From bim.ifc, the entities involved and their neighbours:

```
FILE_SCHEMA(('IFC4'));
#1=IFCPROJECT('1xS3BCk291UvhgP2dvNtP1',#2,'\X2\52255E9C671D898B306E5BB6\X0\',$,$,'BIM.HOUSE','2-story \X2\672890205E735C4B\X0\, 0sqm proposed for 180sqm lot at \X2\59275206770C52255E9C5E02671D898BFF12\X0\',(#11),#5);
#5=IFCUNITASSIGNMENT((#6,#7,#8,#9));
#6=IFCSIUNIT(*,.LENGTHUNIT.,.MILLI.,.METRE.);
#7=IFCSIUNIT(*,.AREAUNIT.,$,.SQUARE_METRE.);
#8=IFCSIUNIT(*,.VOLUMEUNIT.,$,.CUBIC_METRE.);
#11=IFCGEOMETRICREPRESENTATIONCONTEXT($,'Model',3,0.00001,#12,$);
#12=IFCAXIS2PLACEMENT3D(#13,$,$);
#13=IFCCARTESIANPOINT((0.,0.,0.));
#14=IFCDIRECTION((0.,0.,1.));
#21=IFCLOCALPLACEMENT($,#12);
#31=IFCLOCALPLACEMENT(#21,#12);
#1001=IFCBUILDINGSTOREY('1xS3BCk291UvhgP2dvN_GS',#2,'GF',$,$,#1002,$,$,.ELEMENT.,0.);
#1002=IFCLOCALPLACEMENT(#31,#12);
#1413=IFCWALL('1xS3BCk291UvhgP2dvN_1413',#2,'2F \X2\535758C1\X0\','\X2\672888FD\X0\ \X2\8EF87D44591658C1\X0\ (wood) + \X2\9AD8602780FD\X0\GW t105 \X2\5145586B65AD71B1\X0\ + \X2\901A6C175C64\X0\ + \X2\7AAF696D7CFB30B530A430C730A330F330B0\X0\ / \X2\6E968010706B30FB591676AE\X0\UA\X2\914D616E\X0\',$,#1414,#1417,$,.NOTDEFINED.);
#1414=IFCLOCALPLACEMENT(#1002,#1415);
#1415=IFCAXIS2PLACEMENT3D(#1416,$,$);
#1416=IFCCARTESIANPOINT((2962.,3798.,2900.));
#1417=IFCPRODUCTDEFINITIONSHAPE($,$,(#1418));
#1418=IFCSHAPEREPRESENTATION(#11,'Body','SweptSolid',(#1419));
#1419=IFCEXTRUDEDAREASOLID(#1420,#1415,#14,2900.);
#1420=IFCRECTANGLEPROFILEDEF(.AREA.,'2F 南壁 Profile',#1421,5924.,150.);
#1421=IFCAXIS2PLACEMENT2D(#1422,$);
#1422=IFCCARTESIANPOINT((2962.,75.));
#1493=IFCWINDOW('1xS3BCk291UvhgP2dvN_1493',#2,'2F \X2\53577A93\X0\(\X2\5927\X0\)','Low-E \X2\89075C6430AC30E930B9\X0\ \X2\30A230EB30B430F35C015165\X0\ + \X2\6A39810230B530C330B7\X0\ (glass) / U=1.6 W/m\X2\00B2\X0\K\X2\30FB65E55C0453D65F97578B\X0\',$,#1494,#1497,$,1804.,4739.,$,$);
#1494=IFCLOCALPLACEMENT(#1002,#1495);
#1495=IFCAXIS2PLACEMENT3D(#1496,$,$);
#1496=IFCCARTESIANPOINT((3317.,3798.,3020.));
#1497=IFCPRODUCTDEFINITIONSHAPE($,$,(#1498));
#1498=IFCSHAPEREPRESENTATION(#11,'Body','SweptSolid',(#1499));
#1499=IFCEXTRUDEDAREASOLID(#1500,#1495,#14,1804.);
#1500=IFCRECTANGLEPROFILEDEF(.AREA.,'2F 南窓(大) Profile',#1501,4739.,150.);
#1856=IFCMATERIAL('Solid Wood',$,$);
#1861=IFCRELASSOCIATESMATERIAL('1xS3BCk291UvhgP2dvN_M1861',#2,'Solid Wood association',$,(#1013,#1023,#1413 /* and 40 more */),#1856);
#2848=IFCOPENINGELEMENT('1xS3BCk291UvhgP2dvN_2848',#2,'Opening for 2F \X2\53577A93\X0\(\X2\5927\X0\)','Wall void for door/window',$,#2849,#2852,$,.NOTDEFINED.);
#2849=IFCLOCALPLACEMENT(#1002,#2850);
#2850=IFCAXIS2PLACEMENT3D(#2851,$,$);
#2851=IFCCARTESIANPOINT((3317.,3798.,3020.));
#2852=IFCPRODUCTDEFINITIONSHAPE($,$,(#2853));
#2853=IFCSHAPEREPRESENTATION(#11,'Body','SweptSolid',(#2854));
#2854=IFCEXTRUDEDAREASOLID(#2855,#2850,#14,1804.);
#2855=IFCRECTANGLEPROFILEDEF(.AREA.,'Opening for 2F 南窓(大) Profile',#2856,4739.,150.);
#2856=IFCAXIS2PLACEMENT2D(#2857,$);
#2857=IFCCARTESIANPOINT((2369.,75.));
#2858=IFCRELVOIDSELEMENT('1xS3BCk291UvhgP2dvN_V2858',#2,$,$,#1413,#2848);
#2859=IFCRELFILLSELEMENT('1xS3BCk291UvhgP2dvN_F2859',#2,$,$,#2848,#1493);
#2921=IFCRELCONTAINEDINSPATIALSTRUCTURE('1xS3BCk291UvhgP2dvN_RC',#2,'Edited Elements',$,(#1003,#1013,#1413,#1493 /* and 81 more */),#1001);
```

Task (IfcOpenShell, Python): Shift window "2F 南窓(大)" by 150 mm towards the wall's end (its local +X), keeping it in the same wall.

```python
import ifcopenshell
import ifcopenshell.api.geometry
import ifcopenshell.util.placement
import ifcopenshell.util.unit

model = ifcopenshell.open("bim.ifc")
unit_scale = ifcopenshell.util.unit.calculate_unit_scale(model)

window = model.by_id(1493)
opening = window.FillsVoids[0].RelatingOpeningElement
wall = opening.VoidsElements[0].RelatingBuildingElement

wall_matrix = ifcopenshell.util.placement.get_local_placement(wall.ObjectPlacement)
shift = wall_matrix[:3, 0] * 0.15 / unit_scale
before = ifcopenshell.util.placement.get_local_placement(window.ObjectPlacement)[:3, 3].copy()

# The window is not placed relative to its opening, so move both.
for product in (opening, window):
    matrix = ifcopenshell.util.placement.get_local_placement(product.ObjectPlacement)
    matrix[:3, 3] += shift
    ifcopenshell.api.geometry.edit_object_placement(model, product=product, matrix=matrix, is_si=False)

after = ifcopenshell.util.placement.get_local_placement(window.ObjectPlacement)[:3, 3]
print("window moved by", (after - before).round(3) + 0.0)

model.write("bim_updated.ifc")
```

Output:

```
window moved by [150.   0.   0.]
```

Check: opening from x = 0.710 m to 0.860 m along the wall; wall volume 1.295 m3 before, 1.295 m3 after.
